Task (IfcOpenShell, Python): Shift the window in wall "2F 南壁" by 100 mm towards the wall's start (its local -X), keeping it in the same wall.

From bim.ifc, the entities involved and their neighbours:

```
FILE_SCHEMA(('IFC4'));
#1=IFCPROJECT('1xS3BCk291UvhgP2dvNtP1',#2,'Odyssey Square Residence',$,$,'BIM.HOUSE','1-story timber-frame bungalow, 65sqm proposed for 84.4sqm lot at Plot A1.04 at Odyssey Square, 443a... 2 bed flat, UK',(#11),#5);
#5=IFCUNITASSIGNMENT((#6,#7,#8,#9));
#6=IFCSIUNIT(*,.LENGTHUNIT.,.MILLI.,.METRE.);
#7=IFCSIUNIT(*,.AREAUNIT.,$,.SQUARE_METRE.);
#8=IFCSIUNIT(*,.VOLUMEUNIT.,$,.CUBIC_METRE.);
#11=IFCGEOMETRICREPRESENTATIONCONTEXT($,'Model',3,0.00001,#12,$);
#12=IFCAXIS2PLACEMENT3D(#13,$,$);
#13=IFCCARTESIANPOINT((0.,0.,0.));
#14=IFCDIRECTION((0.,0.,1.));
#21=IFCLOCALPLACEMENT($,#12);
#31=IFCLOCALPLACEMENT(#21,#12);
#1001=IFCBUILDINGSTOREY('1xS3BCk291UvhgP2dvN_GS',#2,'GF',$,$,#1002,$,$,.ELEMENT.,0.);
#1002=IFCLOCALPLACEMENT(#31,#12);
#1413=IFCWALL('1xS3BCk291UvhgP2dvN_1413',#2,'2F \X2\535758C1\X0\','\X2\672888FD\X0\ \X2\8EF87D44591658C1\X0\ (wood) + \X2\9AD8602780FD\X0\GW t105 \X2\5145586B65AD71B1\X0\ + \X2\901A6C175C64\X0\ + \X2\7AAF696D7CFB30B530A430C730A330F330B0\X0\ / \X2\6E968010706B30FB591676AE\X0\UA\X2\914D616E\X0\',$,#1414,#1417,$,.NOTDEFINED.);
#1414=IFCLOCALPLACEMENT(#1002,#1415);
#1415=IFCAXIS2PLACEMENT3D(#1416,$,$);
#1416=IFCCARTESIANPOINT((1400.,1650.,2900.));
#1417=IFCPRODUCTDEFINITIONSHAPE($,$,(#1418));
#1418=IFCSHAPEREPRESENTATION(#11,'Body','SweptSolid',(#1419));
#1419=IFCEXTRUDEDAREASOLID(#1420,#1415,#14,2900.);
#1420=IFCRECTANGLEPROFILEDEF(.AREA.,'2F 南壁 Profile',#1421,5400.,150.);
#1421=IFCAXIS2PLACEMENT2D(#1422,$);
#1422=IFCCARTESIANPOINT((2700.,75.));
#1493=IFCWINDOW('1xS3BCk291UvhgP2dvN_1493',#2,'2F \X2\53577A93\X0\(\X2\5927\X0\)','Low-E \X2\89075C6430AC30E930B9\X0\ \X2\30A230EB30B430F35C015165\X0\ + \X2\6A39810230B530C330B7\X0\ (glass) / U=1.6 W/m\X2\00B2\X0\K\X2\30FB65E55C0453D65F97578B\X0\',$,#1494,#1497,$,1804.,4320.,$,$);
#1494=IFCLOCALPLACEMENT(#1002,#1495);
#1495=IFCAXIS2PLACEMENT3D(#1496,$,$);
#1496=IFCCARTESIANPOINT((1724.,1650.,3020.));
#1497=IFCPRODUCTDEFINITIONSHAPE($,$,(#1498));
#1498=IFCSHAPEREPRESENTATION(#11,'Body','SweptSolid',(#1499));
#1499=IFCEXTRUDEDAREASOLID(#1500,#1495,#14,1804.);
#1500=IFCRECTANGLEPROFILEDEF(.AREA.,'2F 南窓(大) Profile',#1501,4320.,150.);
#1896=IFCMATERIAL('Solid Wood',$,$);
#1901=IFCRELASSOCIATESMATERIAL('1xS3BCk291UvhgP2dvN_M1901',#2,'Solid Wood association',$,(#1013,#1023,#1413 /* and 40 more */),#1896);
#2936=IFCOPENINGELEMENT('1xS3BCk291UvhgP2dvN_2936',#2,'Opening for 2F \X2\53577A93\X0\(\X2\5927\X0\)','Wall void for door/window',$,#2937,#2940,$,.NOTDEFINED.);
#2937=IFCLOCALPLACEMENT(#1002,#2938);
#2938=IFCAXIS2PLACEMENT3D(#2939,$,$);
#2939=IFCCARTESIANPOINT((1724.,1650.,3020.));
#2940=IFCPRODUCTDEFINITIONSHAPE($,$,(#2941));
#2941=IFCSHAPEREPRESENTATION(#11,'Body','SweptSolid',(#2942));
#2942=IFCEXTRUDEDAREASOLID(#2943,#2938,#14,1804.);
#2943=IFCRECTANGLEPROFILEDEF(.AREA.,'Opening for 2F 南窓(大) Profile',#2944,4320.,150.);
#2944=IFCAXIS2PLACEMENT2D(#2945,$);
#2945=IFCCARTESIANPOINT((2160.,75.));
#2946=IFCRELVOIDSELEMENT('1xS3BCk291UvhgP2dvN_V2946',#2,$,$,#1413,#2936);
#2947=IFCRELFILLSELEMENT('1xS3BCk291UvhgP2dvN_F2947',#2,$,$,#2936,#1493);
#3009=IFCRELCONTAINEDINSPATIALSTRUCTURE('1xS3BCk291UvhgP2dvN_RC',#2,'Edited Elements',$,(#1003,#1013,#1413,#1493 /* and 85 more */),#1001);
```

```python
import ifcopenshell
import ifcopenshell.api.geometry
import ifcopenshell.util.placement

model = ifcopenshell.open("bim.ifc")

window = model.by_id(1493)
opening = window.FillsVoids[0].RelatingOpeningElement
wall = opening.VoidsElements[0].RelatingBuildingElement

wall_matrix = ifcopenshell.util.placement.get_local_placement(wall.ObjectPlacement)
shift = wall_matrix[:3, 0] * -100.0
before = ifcopenshell.util.placement.get_local_placement(window.ObjectPlacement)[:3, 3].copy()

# The window is not placed relative to its opening, so move both.
for product in (opening, window):
    matrix = ifcopenshell.util.placement.get_local_placement(product.ObjectPlacement)
    matrix[:3, 3] += shift
    ifcopenshell.api.geometry.edit_object_placement(model, product=product, matrix=matrix, is_si=False)

after = ifcopenshell.util.placement.get_local_placement(window.ObjectPlacement)[:3, 3]
print("window moved by", (after - before).round(3) + 0.0)

model.write("bim_v2.ifc")
```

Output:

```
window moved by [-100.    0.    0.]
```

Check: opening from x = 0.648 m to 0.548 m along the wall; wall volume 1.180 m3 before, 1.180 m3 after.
